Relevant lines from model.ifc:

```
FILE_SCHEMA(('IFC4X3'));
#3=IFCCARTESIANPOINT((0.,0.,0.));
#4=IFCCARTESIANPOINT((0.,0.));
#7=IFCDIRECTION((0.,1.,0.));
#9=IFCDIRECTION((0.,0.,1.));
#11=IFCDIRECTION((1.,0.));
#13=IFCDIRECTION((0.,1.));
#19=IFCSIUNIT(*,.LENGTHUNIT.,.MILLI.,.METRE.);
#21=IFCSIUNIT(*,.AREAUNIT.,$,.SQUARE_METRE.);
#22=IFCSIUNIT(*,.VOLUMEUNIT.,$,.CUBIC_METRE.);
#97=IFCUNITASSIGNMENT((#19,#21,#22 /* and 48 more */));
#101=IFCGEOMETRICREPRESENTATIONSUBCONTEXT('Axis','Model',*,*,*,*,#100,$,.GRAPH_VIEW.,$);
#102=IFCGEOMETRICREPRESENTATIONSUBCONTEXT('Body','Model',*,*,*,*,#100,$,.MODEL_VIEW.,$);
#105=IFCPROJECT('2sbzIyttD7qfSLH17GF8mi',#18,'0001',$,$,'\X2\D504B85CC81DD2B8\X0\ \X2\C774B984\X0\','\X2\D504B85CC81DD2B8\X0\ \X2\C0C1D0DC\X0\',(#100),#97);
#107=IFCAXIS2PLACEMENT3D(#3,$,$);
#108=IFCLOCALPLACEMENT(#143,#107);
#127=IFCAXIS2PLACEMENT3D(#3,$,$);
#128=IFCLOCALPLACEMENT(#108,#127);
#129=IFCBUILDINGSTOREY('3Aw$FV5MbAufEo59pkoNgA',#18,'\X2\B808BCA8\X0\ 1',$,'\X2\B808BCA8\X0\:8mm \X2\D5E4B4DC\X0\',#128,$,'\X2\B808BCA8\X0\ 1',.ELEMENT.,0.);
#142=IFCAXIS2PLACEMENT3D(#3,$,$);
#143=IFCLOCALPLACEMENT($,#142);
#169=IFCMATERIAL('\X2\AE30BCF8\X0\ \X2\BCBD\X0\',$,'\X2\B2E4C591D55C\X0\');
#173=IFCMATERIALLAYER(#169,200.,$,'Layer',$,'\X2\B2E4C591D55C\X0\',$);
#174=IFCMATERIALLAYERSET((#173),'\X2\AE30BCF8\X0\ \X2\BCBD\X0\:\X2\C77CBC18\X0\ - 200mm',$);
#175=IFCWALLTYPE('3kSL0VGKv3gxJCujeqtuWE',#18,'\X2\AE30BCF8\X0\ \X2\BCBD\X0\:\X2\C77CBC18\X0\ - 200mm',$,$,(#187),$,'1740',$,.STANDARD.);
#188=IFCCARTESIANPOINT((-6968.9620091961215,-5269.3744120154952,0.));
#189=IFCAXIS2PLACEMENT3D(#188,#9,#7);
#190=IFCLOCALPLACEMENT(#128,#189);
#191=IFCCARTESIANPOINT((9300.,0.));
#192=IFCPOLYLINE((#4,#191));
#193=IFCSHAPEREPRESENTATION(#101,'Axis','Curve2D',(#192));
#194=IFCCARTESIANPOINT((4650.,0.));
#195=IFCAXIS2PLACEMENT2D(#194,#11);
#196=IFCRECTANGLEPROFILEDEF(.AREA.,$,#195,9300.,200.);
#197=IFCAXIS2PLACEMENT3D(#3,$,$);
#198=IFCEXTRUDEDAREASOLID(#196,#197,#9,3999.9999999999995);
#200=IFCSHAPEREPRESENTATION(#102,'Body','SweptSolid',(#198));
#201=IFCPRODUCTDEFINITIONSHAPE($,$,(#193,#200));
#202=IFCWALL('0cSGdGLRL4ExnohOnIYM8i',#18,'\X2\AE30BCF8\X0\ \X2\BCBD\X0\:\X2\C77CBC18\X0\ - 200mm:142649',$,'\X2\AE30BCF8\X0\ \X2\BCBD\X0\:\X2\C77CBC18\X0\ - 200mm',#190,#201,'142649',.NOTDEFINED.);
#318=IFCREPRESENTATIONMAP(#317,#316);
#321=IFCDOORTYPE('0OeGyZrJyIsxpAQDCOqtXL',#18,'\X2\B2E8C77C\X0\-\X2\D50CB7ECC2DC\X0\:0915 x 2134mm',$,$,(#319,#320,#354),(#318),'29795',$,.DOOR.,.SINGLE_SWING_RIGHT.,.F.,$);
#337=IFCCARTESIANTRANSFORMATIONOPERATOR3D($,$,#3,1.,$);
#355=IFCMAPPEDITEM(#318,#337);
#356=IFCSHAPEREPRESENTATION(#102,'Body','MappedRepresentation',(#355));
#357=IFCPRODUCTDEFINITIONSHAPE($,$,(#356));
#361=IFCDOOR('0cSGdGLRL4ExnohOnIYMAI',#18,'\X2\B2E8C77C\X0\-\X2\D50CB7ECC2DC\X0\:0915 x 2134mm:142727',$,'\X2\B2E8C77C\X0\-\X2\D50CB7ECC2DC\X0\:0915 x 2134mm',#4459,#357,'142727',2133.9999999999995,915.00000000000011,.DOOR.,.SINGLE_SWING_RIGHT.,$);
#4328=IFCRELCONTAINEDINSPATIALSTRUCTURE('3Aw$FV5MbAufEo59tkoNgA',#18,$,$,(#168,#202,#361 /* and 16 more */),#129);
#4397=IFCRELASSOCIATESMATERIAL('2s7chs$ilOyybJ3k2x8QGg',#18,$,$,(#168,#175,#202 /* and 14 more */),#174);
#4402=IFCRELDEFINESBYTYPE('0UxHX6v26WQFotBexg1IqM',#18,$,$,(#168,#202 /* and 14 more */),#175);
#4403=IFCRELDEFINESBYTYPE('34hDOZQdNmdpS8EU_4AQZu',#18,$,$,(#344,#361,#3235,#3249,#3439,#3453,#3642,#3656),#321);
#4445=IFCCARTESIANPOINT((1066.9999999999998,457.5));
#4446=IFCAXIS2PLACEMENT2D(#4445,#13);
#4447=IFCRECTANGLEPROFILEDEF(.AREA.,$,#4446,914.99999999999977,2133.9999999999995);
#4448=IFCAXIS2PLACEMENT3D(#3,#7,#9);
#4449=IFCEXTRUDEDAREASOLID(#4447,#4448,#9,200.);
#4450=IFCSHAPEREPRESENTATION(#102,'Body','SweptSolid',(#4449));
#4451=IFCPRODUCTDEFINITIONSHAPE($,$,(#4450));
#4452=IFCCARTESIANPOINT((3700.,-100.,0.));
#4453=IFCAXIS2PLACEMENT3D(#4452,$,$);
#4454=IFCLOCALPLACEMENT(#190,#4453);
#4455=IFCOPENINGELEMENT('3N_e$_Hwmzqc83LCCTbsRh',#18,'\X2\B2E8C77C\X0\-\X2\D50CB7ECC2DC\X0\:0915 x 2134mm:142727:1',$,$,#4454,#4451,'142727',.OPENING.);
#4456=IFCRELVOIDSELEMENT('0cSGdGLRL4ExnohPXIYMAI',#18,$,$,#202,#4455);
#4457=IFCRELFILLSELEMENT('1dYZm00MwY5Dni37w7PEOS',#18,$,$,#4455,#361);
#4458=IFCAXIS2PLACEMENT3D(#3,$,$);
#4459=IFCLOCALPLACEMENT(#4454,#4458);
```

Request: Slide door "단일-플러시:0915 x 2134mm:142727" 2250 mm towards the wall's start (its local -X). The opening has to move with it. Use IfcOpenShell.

```python
import ifcopenshell
import ifcopenshell.api.geometry
import ifcopenshell.util.placement
import ifcopenshell.util.unit

model = ifcopenshell.open("model.ifc")
unit_scale = ifcopenshell.util.unit.calculate_unit_scale(model)

door = model.by_id(361)
opening = door.FillsVoids[0].RelatingOpeningElement
wall = opening.VoidsElements[0].RelatingBuildingElement

wall_matrix = ifcopenshell.util.placement.get_local_placement(wall.ObjectPlacement)
shift = wall_matrix[:3, 0] * -2.25 / unit_scale
before = ifcopenshell.util.placement.get_local_placement(door.ObjectPlacement)[:3, 3].copy()

# The door is placed relative to its opening, so it follows when the opening moves.
matrix = ifcopenshell.util.placement.get_local_placement(opening.ObjectPlacement)
matrix[:3, 3] += shift
ifcopenshell.api.geometry.edit_object_placement(
    model, product=opening, matrix=matrix, is_si=False, should_transform_children=True
)

after = ifcopenshell.util.placement.get_local_placement(door.ObjectPlacement)[:3, 3]
print("door moved by", (after - before).round(3) + 0.0)

model.write("model_v2.ifc")
```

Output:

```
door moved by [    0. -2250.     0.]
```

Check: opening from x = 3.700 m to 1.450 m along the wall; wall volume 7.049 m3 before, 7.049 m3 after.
